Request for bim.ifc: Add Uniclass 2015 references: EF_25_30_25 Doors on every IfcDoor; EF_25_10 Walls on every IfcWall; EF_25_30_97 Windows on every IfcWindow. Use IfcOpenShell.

First a look at what the model holds.

```python
import ifcopenshell

model = ifcopenshell.open("bim.ifc")
print(model.schema)
print("classifications:", [c.Name for c in model.by_type("IfcClassification")])
for ifc_class in ("IfcDoor", "IfcRoof", "IfcStair", "IfcWall", "IfcWindow"):
    print(ifc_class, len(model.by_type(ifc_class)))
```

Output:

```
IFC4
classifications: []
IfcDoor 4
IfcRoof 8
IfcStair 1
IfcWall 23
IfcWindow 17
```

```python
import ifcopenshell
import ifcopenshell.api.classification

model = ifcopenshell.open("bim.ifc")

system = ifcopenshell.api.classification.add_classification(model, classification="Uniclass 2015")

codes = {
    "IfcDoor": ("EF_25_30_25", "Doors"),
    "IfcWall": ("EF_25_10", "Walls"),
    "IfcWindow": ("EF_25_30_97", "Windows"),
}
for ifc_class, (code, name) in codes.items():
    products = model.by_type(ifc_class)
    ifcopenshell.api.classification.add_reference(
        model, products=products, classification=system, identification=code, name=name
    )
    print(code, len(products))

model.write("bim_updated.ifc")
```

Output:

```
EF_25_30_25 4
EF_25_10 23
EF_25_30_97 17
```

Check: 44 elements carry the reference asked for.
